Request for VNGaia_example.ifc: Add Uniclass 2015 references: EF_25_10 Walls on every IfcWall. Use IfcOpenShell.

First a look at what the model holds.

```python
import ifcopenshell

model = ifcopenshell.open("VNGaia_example.ifc")
print(model.schema)
print("classifications:", [c.Name for c in model.by_type("IfcClassification")])
for ifc_class in ("IfcDoor", "IfcRoof", "IfcStair", "IfcWall", "IfcWindow"):
    print(ifc_class, len(model.by_type(ifc_class)))
```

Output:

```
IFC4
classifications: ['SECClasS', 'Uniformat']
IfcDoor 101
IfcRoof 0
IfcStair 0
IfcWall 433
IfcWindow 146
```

```python
import ifcopenshell
import ifcopenshell.api.classification

model = ifcopenshell.open("VNGaia_example.ifc")

system = ifcopenshell.api.classification.add_classification(model, classification="Uniclass 2015")

codes = {
    "IfcWall": ("EF_25_10", "Walls"),
}
for ifc_class, (code, name) in codes.items():
    products = model.by_type(ifc_class)
    ifcopenshell.api.classification.add_reference(
        model, products=products, classification=system, identification=code, name=name
    )
    print(code, len(products))

model.write("VNGaia_example_rev.ifc")
```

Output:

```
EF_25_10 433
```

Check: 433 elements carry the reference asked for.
